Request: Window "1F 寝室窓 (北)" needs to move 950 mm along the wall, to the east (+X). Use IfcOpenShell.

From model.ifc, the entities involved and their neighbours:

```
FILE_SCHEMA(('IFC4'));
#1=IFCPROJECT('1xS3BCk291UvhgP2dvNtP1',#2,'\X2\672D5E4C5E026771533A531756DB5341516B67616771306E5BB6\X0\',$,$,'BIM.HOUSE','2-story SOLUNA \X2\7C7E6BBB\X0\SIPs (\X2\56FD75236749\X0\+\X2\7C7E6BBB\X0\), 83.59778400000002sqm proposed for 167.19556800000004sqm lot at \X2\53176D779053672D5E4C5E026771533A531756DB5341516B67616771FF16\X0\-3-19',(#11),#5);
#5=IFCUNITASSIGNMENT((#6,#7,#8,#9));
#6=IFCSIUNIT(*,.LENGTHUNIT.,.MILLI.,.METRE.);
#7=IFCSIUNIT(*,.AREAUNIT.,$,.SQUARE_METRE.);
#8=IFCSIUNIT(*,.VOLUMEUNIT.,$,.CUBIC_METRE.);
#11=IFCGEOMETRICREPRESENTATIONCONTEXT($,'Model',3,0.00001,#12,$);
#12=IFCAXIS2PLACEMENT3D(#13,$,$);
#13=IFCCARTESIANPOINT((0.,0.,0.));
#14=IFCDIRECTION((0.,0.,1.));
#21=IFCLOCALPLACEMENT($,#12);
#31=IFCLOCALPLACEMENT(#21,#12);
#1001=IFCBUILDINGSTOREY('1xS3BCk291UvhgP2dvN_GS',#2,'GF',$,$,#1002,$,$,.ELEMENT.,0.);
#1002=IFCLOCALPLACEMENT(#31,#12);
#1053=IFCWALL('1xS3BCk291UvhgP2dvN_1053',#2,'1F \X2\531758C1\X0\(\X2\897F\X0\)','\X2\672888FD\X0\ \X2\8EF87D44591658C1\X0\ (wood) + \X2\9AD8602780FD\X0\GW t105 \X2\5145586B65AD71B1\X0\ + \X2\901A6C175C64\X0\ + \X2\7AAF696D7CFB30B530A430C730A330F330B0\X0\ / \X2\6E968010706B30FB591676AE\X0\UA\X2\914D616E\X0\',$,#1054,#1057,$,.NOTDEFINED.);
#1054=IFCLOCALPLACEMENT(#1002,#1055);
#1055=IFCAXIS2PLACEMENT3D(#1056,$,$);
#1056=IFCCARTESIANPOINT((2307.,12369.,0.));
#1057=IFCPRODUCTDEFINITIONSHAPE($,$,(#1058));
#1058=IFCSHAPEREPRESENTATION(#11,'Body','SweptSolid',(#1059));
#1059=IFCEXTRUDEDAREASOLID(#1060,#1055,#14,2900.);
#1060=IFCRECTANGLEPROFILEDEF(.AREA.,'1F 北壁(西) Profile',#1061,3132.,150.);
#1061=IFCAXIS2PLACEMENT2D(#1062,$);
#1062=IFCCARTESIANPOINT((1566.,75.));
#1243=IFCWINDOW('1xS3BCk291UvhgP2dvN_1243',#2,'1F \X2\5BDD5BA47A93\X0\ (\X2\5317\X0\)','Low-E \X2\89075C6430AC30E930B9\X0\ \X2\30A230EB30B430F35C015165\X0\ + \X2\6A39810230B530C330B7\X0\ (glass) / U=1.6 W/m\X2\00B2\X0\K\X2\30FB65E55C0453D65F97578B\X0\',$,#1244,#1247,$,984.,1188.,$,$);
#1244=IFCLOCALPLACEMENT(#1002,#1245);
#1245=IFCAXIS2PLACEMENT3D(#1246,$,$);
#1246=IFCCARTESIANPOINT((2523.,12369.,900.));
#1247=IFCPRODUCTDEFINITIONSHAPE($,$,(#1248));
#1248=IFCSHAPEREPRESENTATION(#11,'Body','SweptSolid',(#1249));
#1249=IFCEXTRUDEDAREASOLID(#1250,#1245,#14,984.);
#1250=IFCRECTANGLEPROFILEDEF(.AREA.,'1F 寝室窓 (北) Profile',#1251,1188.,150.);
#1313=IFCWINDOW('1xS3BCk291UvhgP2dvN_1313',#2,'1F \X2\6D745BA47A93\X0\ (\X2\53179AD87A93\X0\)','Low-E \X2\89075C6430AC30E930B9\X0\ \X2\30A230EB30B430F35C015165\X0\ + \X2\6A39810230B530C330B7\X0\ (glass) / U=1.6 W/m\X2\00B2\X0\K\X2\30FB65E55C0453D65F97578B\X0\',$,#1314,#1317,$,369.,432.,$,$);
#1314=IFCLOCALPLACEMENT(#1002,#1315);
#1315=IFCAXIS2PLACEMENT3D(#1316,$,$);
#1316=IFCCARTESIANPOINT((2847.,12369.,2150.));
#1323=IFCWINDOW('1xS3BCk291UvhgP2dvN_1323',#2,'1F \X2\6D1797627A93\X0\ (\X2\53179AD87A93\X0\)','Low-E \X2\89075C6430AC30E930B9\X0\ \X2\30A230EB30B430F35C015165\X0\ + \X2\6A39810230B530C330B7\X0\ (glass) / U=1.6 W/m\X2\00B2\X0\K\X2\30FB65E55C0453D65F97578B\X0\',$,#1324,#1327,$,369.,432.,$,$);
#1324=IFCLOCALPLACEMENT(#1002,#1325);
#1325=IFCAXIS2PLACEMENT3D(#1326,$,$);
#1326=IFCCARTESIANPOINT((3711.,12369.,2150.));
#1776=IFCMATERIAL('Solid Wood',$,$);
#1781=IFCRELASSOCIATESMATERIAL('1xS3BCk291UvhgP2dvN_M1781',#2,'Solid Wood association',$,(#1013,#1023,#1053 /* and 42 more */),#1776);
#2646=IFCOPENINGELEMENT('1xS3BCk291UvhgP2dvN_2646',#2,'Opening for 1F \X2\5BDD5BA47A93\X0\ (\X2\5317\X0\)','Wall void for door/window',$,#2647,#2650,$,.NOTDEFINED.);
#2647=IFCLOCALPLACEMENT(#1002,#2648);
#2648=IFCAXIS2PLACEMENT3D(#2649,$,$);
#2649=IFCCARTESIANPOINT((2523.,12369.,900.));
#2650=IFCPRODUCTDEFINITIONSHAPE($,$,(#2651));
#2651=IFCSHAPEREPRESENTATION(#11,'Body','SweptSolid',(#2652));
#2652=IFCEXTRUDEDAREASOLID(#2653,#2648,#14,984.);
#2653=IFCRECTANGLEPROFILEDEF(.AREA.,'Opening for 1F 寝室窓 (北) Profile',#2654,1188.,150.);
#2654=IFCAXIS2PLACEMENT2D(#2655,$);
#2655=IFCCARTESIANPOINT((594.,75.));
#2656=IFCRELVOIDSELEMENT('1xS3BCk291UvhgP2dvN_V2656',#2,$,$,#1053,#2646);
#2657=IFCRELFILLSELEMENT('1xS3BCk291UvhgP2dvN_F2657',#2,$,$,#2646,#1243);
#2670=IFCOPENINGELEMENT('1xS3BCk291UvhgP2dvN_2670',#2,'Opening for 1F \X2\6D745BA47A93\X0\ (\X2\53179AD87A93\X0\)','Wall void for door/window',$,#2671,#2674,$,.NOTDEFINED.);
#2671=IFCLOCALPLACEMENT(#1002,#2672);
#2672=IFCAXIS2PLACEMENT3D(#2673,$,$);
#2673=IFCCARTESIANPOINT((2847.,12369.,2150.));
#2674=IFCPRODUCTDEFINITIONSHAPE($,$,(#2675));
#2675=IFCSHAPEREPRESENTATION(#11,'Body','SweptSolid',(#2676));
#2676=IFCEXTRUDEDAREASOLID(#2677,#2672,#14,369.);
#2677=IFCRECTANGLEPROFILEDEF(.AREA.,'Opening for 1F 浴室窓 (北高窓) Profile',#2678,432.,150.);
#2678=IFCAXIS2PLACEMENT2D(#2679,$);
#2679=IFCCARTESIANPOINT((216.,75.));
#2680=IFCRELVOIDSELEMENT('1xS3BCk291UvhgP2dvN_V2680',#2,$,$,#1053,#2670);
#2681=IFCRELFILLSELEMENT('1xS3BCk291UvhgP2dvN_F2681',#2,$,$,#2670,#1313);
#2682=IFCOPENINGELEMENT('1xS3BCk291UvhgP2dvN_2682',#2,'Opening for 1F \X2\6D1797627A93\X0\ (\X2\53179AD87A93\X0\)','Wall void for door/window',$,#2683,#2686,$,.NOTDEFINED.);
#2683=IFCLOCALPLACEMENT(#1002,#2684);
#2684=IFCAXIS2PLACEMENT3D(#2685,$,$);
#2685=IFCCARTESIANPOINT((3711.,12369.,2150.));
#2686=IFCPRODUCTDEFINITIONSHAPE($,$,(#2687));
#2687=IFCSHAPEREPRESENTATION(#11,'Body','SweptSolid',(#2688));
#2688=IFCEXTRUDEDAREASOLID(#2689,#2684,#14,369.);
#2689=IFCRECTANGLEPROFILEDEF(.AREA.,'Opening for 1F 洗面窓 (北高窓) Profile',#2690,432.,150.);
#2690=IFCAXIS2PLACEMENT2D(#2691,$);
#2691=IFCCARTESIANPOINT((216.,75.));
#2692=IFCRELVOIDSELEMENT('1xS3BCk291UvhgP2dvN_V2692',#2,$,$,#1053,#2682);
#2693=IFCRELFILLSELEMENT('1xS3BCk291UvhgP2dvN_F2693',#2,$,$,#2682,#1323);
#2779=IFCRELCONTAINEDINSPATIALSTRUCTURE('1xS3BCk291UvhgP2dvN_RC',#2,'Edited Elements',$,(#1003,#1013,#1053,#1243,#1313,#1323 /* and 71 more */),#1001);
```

```python
import ifcopenshell
import ifcopenshell.api.geometry
import ifcopenshell.util.placement
import ifcopenshell.util.unit

model = ifcopenshell.open("model.ifc")
unit_scale = ifcopenshell.util.unit.calculate_unit_scale(model)

window = model.by_guid("1xS3BCk291UvhgP2dvN_1243")
opening = window.FillsVoids[0].RelatingOpeningElement
wall = opening.VoidsElements[0].RelatingBuildingElement

wall_matrix = ifcopenshell.util.placement.get_local_placement(wall.ObjectPlacement)
shift = wall_matrix[:3, 0] * 0.95 / unit_scale
before = ifcopenshell.util.placement.get_local_placement(window.ObjectPlacement)[:3, 3].copy()

# The window is not placed relative to its opening, so move both.
for product in (opening, window):
    matrix = ifcopenshell.util.placement.get_local_placement(product.ObjectPlacement)
    matrix[:3, 3] += shift
    ifcopenshell.api.geometry.edit_object_placement(model, product=product, matrix=matrix, is_si=False)

after = ifcopenshell.util.placement.get_local_placement(window.ObjectPlacement)[:3, 3]
print("window moved by", (after - before).round(3) + 0.0)

model.write("model_edited.ifc")
```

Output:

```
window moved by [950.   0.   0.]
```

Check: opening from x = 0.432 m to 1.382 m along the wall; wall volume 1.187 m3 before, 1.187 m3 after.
